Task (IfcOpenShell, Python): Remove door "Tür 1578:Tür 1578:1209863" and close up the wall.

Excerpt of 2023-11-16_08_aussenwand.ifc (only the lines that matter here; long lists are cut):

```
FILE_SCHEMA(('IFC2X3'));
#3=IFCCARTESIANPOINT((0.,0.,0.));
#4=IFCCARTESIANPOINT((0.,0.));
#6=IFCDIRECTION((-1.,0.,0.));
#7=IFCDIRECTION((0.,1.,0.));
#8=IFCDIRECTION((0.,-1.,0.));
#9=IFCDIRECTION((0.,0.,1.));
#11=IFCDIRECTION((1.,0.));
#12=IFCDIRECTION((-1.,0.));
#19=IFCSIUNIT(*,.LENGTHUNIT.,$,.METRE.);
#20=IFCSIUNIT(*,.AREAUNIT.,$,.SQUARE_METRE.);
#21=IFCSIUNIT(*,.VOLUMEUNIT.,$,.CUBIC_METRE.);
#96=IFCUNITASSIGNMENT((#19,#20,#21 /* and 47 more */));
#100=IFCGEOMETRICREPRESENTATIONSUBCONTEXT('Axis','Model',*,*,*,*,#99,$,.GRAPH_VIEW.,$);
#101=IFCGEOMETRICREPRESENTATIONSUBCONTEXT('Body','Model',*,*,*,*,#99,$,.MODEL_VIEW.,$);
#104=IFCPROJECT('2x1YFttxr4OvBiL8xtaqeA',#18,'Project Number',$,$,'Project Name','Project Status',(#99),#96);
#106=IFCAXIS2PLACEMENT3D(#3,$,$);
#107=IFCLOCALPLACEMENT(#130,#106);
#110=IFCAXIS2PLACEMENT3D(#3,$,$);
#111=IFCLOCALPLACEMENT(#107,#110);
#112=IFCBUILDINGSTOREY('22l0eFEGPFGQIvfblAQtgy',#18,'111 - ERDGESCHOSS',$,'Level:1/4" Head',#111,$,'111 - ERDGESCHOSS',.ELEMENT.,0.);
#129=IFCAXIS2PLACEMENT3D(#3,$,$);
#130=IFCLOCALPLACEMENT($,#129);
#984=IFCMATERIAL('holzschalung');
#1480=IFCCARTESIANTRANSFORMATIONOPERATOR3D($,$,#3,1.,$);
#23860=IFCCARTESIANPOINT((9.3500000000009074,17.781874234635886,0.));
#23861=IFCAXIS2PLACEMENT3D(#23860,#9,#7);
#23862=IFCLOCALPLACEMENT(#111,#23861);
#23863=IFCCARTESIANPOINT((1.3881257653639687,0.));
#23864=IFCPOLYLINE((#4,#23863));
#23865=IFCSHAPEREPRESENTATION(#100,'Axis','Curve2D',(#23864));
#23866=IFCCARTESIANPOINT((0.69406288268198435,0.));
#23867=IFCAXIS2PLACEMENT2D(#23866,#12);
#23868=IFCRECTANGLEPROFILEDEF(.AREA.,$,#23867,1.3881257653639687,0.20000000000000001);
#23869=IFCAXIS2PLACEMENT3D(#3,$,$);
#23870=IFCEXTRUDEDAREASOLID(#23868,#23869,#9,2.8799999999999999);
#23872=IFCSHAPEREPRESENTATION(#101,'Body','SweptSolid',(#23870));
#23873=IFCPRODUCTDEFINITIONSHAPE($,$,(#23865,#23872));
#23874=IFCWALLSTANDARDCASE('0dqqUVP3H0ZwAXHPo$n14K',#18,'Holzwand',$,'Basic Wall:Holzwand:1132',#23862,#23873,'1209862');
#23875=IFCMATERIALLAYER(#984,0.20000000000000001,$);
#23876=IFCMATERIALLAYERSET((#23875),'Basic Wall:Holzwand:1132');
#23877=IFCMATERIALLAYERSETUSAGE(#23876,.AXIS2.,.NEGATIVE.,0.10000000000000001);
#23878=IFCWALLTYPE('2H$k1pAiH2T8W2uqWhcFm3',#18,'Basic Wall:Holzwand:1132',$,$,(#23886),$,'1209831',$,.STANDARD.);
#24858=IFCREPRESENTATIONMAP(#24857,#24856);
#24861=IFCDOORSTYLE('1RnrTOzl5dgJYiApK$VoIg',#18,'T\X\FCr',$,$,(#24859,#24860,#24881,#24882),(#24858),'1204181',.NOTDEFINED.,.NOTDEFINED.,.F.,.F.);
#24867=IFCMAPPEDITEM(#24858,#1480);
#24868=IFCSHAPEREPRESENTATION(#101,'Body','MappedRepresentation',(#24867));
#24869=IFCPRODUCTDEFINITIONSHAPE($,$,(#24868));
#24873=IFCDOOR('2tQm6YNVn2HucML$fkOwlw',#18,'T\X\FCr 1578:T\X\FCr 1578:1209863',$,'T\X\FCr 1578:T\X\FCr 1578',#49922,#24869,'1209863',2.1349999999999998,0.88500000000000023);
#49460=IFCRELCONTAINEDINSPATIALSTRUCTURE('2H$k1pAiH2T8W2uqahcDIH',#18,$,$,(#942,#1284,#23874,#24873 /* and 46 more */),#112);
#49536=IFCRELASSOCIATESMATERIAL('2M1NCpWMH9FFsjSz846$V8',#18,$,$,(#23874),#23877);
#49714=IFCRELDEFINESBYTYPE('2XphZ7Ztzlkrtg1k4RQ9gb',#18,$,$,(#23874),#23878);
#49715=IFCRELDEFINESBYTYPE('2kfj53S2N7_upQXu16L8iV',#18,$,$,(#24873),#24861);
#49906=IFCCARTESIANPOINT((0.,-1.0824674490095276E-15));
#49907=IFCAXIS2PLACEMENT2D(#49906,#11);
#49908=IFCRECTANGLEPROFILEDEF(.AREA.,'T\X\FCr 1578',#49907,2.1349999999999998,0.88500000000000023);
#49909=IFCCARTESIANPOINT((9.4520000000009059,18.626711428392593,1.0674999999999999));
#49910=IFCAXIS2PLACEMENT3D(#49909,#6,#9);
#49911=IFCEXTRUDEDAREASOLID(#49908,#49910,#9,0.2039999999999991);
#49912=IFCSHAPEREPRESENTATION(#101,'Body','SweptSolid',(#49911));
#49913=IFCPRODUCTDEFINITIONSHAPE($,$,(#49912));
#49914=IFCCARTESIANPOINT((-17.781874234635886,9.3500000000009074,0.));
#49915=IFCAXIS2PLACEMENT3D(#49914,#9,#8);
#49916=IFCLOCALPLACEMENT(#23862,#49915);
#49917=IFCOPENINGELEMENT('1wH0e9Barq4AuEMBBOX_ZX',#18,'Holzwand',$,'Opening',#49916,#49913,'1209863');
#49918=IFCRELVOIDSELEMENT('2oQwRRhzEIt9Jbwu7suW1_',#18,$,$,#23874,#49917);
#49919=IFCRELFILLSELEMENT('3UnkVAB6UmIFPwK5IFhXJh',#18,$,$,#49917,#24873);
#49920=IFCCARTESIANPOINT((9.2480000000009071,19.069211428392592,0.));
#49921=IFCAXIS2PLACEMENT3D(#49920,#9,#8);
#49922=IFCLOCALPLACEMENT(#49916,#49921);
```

```python
import ifcopenshell
import ifcopenshell.api.feature
import ifcopenshell.api.root
import ifcopenshell.geom
import ifcopenshell.util.shape

model = ifcopenshell.open("2023-11-16_08_aussenwand.ifc")
settings = ifcopenshell.geom.settings()


def volume(element):
    """Net volume in cubic metres, openings subtracted."""
    shape = ifcopenshell.geom.create_shape(settings, element)
    return ifcopenshell.util.shape.get_volume(shape.geometry)


door = model.by_guid("2tQm6YNVn2HucML$fkOwlw")
opening = door.FillsVoids[0].RelatingOpeningElement
wall = opening.VoidsElements[0].RelatingBuildingElement
before = volume(wall)

ifcopenshell.api.root.remove_product(model, product=door)
ifcopenshell.api.feature.remove_feature(model, feature=opening)

after = volume(wall)

print(f"wall volume {before:.3f} -> {after:.3f} m3")

model.write("2023-11-16_08_aussenwand_rev.ifc")
```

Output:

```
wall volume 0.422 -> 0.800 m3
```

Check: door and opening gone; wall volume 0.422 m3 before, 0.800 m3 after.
